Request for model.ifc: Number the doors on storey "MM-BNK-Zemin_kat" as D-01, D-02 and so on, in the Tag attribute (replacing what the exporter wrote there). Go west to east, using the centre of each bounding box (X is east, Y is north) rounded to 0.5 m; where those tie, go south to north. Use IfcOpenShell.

First a look at what the model holds.

```python
import ifcopenshell
import ifcopenshell.util.element
import ifcopenshell.util.placement

model = ifcopenshell.open("model.ifc")
print(model.schema)
storey = next(s for s in model.by_type("IfcBuildingStorey") if s.Name == "MM-BNK-Zemin_kat")
doors = [e for e in ifcopenshell.util.element.get_decomposition(storey) if e.is_a("IfcDoor")]
for e in sorted(doors, key=lambda e: e.id()):
    origin = ifcopenshell.util.placement.get_local_placement(e.ObjectPlacement)[:3, 3]
    print(e.id(), e.Tag, e.Name, origin.round(2) + 0.0, sep=" | ")
```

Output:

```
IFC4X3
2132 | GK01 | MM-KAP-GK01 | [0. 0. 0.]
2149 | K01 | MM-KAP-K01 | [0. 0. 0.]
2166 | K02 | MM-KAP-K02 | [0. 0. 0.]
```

```python
import ifcopenshell
import ifcopenshell.geom
import ifcopenshell.util.element
import ifcopenshell.util.shape

model = ifcopenshell.open("model.ifc")
settings = ifcopenshell.geom.settings()
settings.set("use-world-coords", True)


def centre(element):
    shape = ifcopenshell.geom.create_shape(settings, element)
    return ifcopenshell.util.shape.get_bbox_centroid(shape.geometry)


storey = next(s for s in model.by_type("IfcBuildingStorey") if s.Name == "MM-BNK-Zemin_kat")
doors = [e for e in ifcopenshell.util.element.get_decomposition(storey) if e.is_a("IfcDoor")]

# Insertion points can sit at a corner or the storey origin, so sort by the geometry (in metres).
centres = {e: centre(e) for e in doors}
doors.sort(key=lambda e: (round(centres[e][0] / 0.5), centres[e][1]))

for i, e in enumerate(doors, start=1):
    number = f"D-{i:02d}"
    e.Tag = number
    print(e.id(), number)

model.write("model_v2.ifc")
```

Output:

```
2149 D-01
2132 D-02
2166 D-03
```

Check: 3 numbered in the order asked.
